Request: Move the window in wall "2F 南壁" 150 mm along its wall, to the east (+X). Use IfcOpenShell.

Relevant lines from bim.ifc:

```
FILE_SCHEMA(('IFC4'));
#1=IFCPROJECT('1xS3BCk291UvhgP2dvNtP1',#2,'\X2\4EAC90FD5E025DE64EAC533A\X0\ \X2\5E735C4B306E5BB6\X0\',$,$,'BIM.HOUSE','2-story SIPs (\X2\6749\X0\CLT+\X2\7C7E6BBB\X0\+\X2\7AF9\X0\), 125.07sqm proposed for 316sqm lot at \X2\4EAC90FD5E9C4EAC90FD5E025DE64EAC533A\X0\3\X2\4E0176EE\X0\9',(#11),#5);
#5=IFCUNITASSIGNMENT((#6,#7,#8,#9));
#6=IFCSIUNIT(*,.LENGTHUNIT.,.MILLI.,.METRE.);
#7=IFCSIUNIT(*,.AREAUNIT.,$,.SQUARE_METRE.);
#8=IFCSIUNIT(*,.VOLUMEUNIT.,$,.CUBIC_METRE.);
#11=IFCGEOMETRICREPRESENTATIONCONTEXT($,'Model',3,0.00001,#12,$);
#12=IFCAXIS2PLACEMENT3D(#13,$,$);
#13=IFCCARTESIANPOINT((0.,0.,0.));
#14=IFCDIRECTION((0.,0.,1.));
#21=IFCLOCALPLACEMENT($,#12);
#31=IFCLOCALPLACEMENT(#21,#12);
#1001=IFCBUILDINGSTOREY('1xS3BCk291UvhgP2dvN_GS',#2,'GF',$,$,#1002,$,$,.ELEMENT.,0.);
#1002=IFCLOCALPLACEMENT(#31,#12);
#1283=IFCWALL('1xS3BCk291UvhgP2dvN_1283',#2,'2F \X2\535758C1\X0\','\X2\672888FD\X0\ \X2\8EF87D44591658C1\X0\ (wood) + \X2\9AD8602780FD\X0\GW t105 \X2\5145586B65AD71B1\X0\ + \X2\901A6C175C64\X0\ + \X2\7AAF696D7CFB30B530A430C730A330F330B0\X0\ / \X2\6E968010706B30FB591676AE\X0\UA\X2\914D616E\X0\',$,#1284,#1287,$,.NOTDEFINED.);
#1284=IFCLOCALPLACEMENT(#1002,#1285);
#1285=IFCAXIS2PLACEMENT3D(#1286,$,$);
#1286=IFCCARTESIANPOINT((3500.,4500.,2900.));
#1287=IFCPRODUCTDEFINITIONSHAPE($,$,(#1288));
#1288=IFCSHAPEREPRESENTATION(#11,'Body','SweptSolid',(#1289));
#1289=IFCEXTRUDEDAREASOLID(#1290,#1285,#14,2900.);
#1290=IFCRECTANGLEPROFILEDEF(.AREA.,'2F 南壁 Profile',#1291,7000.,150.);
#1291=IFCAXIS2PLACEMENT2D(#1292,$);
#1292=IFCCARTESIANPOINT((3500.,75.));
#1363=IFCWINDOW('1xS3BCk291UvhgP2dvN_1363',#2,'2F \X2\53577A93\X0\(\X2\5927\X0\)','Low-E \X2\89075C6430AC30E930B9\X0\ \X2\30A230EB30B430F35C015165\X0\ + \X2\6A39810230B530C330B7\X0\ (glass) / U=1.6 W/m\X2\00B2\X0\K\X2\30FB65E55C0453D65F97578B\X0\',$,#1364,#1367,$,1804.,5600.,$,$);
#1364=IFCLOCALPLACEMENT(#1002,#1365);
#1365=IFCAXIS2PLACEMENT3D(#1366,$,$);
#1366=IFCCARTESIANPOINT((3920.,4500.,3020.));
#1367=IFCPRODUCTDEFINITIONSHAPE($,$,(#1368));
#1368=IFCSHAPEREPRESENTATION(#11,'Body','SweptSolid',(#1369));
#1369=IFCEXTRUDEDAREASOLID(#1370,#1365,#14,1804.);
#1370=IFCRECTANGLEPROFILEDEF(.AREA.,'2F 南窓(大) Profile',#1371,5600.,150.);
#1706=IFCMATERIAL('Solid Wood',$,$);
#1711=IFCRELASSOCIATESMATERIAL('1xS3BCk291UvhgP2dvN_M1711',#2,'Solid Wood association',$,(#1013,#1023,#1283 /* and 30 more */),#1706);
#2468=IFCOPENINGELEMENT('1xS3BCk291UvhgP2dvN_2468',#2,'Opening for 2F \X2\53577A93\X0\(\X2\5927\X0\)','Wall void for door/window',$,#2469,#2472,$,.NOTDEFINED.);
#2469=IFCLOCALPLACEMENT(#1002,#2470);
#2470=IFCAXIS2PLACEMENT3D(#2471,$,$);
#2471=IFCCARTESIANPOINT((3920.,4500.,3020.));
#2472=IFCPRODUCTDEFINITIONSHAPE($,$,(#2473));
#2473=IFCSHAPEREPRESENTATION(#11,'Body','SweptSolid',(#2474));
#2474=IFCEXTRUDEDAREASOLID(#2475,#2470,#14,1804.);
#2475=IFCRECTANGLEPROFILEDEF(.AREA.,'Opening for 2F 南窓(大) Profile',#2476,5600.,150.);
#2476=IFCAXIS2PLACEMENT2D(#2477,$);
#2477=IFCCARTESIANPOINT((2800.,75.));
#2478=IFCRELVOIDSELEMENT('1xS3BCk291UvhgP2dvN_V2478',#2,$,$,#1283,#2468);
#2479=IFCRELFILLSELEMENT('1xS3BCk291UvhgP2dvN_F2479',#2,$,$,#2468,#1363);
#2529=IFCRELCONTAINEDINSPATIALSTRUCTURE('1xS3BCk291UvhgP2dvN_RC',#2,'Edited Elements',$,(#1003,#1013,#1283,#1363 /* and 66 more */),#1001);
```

```python
import ifcopenshell
import ifcopenshell.api.geometry
import ifcopenshell.util.placement
import ifcopenshell.util.unit

model = ifcopenshell.open("bim.ifc")
unit_scale = ifcopenshell.util.unit.calculate_unit_scale(model)

window = model.by_guid("1xS3BCk291UvhgP2dvN_1363")
opening = window.FillsVoids[0].RelatingOpeningElement
wall = opening.VoidsElements[0].RelatingBuildingElement

wall_matrix = ifcopenshell.util.placement.get_local_placement(wall.ObjectPlacement)
shift = wall_matrix[:3, 0] * 0.15 / unit_scale
before = ifcopenshell.util.placement.get_local_placement(window.ObjectPlacement)[:3, 3].copy()

# The window is not placed relative to its opening, so move both.
for product in (opening, window):
    matrix = ifcopenshell.util.placement.get_local_placement(product.ObjectPlacement)
    matrix[:3, 3] += shift
    ifcopenshell.api.geometry.edit_object_placement(model, product=product, matrix=matrix, is_si=False)

after = ifcopenshell.util.placement.get_local_placement(window.ObjectPlacement)[:3, 3]
print("window moved by", (after - before).round(3) + 0.0)

model.write("bim_updated.ifc")
```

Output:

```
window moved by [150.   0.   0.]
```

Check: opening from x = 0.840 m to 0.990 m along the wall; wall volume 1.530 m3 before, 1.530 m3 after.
